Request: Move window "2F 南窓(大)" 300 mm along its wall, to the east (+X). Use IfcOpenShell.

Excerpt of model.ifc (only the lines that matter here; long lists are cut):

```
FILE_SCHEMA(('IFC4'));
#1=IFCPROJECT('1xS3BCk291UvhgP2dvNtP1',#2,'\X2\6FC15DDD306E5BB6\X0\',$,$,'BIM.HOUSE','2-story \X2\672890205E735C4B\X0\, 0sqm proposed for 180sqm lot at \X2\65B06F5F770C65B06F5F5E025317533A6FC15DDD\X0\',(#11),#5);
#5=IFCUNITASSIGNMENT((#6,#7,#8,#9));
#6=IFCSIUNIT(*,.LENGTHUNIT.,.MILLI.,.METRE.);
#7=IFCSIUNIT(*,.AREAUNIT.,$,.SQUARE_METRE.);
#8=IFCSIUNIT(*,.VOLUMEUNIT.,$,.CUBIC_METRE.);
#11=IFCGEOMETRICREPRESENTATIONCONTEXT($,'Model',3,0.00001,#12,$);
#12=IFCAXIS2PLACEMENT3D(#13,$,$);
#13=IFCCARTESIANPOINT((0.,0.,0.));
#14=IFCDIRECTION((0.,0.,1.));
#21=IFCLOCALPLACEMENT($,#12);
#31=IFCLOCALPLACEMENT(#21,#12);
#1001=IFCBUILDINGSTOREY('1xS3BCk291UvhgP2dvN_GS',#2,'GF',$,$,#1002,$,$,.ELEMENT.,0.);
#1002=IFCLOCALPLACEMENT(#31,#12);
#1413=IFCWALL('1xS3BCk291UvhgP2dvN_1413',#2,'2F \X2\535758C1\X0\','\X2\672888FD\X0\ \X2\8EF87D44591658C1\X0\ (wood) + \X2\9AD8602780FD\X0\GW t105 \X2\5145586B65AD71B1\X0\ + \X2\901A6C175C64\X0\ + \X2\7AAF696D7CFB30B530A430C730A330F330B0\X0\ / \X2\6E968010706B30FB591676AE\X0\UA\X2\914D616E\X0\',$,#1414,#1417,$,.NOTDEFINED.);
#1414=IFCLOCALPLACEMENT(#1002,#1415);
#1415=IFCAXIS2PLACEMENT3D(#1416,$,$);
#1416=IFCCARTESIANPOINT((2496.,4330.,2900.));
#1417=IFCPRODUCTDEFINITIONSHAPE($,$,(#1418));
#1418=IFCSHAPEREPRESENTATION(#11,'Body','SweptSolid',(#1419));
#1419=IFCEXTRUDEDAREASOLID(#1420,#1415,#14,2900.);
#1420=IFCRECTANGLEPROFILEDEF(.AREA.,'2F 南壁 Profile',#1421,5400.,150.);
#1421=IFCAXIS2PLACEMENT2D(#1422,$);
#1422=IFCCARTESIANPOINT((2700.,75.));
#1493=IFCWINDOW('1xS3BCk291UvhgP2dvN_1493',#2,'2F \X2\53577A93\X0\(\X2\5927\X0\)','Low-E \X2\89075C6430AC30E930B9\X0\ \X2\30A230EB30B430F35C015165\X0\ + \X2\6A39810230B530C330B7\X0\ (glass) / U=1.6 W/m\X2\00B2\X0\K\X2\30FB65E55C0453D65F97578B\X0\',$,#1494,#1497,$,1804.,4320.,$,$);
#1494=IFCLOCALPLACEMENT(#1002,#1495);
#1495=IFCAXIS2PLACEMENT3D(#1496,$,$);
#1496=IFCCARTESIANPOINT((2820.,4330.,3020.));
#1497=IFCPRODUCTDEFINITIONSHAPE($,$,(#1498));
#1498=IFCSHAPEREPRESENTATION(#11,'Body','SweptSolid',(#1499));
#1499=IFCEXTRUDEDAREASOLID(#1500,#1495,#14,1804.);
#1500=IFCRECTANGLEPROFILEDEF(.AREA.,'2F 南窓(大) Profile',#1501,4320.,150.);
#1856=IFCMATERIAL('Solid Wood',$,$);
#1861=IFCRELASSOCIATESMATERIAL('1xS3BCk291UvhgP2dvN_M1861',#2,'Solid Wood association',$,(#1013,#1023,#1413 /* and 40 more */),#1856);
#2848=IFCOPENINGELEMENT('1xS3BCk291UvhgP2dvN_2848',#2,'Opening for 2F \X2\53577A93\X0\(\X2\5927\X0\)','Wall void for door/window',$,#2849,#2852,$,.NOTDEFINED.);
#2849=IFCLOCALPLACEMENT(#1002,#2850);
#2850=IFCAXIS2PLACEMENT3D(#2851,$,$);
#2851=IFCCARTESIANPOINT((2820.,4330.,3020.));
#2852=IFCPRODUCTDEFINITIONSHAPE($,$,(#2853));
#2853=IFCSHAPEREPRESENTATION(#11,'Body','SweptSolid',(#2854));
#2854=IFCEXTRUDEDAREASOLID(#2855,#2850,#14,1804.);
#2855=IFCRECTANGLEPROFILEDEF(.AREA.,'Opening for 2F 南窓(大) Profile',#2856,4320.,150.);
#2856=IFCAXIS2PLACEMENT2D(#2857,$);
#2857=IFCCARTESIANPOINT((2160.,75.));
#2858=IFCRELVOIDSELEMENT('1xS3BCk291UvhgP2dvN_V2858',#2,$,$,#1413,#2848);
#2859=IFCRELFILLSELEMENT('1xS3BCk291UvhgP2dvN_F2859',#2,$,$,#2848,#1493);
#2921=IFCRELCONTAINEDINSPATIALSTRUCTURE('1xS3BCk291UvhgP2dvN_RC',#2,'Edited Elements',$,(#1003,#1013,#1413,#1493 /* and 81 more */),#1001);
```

```python
import ifcopenshell
import ifcopenshell.api.geometry
import ifcopenshell.util.placement
import ifcopenshell.util.unit

model = ifcopenshell.open("model.ifc")
unit_scale = ifcopenshell.util.unit.calculate_unit_scale(model)

window = model.by_guid("1xS3BCk291UvhgP2dvN_1493")
opening = window.FillsVoids[0].RelatingOpeningElement
wall = opening.VoidsElements[0].RelatingBuildingElement

wall_matrix = ifcopenshell.util.placement.get_local_placement(wall.ObjectPlacement)
shift = wall_matrix[:3, 0] * 0.3 / unit_scale
before = ifcopenshell.util.placement.get_local_placement(window.ObjectPlacement)[:3, 3].copy()

# The window is not placed relative to its opening, so move both.
for product in (opening, window):
    matrix = ifcopenshell.util.placement.get_local_placement(product.ObjectPlacement)
    matrix[:3, 3] += shift
    ifcopenshell.api.geometry.edit_object_placement(model, product=product, matrix=matrix, is_si=False)

after = ifcopenshell.util.placement.get_local_placement(window.ObjectPlacement)[:3, 3]
print("window moved by", (after - before).round(3) + 0.0)

model.write("model_v2.ifc")
```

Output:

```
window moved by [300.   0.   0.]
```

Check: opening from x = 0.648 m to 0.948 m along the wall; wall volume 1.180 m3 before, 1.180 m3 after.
